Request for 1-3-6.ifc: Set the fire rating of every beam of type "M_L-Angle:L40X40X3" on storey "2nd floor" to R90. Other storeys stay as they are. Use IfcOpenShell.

First a look at what the model holds.

```python
import ifcopenshell
import ifcopenshell.util.element

model = ifcopenshell.open("1-3-6.ifc")
print(model.schema)
storey = next(s for s in model.by_type("IfcBuildingStorey") if s.Name == "2nd floor")
beams = [e for e in ifcopenshell.util.element.get_decomposition(storey) if e.is_a("IfcBeam")]
seen = {}
for e in beams:
    element_type = ifcopenshell.util.element.get_type(e)
    key = (element_type.Name if element_type != e and element_type else None, ifcopenshell.util.element.get_pset(e, "Pset_BeamCommon", "FireRating"))
    seen[key] = seen.get(key, 0) + 1
for (name, value), count in sorted(seen.items(), key=str):
    print(count, "x", name, "|", value)
```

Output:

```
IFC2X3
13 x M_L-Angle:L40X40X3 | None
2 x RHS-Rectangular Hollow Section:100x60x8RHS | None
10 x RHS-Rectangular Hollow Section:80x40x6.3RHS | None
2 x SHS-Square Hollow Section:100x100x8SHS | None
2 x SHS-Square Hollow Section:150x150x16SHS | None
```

```python
import ifcopenshell
import ifcopenshell.api.pset
import ifcopenshell.util.element

model = ifcopenshell.open("1-3-6.ifc")

storey = next(s for s in model.by_type("IfcBuildingStorey") if s.Name == "2nd floor")
beams = [e for e in ifcopenshell.util.element.get_decomposition(storey) if e.is_a("IfcBeam")]

count = 0
for e in beams:
    element_type = ifcopenshell.util.element.get_type(e)
    if element_type in (None, e) or element_type.Name != "M_L-Angle:L40X40X3":
        continue
    # add_pset returns the element's existing set when there is one.
    pset = ifcopenshell.api.pset.add_pset(model, product=e, name="Pset_BeamCommon")
    ifcopenshell.api.pset.edit_pset(model, pset=pset, properties={"FireRating": "R90"})
    count += 1

print(count, "beams updated")

model.write("1-3-6_rev.ifc")
```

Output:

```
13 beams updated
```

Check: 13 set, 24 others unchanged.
